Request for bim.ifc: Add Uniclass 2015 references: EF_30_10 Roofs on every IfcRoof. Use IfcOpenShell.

First a look at what the model holds.

```python
import ifcopenshell

model = ifcopenshell.open("bim.ifc")
print(model.schema)
print("classifications:", [c.Name for c in model.by_type("IfcClassification")])
for ifc_class in ("IfcDoor", "IfcRoof", "IfcStair", "IfcWall", "IfcWindow"):
    print(ifc_class, len(model.by_type(ifc_class)))
```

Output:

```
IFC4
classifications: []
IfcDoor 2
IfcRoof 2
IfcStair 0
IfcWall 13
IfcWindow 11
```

```python
import ifcopenshell
import ifcopenshell.api.classification

model = ifcopenshell.open("bim.ifc")

system = ifcopenshell.api.classification.add_classification(model, classification="Uniclass 2015")

codes = {
    "IfcRoof": ("EF_30_10", "Roofs"),
}
for ifc_class, (code, name) in codes.items():
    products = model.by_type(ifc_class)
    ifcopenshell.api.classification.add_reference(
        model, products=products, classification=system, identification=code, name=name
    )
    print(code, len(products))

model.write("bim_v2.ifc")
```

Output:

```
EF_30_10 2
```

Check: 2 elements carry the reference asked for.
